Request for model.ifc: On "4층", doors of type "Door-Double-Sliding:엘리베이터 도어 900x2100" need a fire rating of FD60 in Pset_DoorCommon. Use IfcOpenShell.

First a look at what the model holds.

```python
import ifcopenshell
import ifcopenshell.util.element

model = ifcopenshell.open("model.ifc")
print(model.schema)
storey = next(s for s in model.by_type("IfcBuildingStorey") if s.Name == "4층")
doors = [e for e in ifcopenshell.util.element.get_decomposition(storey) if e.is_a("IfcDoor")]
seen = {}
for e in doors:
    element_type = ifcopenshell.util.element.get_type(e)
    key = (element_type.Name if element_type != e and element_type else None, ifcopenshell.util.element.get_pset(e, "Pset_DoorCommon", "FireRating"))
    seen[key] = seen.get(key, 0) + 1
for (name, value), count in sorted(seen.items(), key=str):
    print(count, "x", name, "|", value)
```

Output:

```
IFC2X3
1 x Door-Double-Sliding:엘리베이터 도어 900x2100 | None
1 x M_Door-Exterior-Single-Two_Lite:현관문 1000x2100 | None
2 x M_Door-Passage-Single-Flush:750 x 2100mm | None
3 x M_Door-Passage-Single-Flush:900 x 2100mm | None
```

```python
import ifcopenshell
import ifcopenshell.api.pset
import ifcopenshell.util.element

model = ifcopenshell.open("model.ifc")

storey = next(s for s in model.by_type("IfcBuildingStorey") if s.Name == "4층")
doors = [e for e in ifcopenshell.util.element.get_decomposition(storey) if e.is_a("IfcDoor")]

count = 0
for e in doors:
    element_type = ifcopenshell.util.element.get_type(e)
    if element_type in (None, e) or element_type.Name != "Door-Double-Sliding:엘리베이터 도어 900x2100":
        continue
    # add_pset returns the element's existing set when there is one.
    pset = ifcopenshell.api.pset.add_pset(model, product=e, name="Pset_DoorCommon")
    ifcopenshell.api.pset.edit_pset(model, pset=pset, properties={"FireRating": "FD60"})
    count += 1

print(count, "doors updated")

model.write("model-out.ifc")
```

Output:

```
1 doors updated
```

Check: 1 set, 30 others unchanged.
